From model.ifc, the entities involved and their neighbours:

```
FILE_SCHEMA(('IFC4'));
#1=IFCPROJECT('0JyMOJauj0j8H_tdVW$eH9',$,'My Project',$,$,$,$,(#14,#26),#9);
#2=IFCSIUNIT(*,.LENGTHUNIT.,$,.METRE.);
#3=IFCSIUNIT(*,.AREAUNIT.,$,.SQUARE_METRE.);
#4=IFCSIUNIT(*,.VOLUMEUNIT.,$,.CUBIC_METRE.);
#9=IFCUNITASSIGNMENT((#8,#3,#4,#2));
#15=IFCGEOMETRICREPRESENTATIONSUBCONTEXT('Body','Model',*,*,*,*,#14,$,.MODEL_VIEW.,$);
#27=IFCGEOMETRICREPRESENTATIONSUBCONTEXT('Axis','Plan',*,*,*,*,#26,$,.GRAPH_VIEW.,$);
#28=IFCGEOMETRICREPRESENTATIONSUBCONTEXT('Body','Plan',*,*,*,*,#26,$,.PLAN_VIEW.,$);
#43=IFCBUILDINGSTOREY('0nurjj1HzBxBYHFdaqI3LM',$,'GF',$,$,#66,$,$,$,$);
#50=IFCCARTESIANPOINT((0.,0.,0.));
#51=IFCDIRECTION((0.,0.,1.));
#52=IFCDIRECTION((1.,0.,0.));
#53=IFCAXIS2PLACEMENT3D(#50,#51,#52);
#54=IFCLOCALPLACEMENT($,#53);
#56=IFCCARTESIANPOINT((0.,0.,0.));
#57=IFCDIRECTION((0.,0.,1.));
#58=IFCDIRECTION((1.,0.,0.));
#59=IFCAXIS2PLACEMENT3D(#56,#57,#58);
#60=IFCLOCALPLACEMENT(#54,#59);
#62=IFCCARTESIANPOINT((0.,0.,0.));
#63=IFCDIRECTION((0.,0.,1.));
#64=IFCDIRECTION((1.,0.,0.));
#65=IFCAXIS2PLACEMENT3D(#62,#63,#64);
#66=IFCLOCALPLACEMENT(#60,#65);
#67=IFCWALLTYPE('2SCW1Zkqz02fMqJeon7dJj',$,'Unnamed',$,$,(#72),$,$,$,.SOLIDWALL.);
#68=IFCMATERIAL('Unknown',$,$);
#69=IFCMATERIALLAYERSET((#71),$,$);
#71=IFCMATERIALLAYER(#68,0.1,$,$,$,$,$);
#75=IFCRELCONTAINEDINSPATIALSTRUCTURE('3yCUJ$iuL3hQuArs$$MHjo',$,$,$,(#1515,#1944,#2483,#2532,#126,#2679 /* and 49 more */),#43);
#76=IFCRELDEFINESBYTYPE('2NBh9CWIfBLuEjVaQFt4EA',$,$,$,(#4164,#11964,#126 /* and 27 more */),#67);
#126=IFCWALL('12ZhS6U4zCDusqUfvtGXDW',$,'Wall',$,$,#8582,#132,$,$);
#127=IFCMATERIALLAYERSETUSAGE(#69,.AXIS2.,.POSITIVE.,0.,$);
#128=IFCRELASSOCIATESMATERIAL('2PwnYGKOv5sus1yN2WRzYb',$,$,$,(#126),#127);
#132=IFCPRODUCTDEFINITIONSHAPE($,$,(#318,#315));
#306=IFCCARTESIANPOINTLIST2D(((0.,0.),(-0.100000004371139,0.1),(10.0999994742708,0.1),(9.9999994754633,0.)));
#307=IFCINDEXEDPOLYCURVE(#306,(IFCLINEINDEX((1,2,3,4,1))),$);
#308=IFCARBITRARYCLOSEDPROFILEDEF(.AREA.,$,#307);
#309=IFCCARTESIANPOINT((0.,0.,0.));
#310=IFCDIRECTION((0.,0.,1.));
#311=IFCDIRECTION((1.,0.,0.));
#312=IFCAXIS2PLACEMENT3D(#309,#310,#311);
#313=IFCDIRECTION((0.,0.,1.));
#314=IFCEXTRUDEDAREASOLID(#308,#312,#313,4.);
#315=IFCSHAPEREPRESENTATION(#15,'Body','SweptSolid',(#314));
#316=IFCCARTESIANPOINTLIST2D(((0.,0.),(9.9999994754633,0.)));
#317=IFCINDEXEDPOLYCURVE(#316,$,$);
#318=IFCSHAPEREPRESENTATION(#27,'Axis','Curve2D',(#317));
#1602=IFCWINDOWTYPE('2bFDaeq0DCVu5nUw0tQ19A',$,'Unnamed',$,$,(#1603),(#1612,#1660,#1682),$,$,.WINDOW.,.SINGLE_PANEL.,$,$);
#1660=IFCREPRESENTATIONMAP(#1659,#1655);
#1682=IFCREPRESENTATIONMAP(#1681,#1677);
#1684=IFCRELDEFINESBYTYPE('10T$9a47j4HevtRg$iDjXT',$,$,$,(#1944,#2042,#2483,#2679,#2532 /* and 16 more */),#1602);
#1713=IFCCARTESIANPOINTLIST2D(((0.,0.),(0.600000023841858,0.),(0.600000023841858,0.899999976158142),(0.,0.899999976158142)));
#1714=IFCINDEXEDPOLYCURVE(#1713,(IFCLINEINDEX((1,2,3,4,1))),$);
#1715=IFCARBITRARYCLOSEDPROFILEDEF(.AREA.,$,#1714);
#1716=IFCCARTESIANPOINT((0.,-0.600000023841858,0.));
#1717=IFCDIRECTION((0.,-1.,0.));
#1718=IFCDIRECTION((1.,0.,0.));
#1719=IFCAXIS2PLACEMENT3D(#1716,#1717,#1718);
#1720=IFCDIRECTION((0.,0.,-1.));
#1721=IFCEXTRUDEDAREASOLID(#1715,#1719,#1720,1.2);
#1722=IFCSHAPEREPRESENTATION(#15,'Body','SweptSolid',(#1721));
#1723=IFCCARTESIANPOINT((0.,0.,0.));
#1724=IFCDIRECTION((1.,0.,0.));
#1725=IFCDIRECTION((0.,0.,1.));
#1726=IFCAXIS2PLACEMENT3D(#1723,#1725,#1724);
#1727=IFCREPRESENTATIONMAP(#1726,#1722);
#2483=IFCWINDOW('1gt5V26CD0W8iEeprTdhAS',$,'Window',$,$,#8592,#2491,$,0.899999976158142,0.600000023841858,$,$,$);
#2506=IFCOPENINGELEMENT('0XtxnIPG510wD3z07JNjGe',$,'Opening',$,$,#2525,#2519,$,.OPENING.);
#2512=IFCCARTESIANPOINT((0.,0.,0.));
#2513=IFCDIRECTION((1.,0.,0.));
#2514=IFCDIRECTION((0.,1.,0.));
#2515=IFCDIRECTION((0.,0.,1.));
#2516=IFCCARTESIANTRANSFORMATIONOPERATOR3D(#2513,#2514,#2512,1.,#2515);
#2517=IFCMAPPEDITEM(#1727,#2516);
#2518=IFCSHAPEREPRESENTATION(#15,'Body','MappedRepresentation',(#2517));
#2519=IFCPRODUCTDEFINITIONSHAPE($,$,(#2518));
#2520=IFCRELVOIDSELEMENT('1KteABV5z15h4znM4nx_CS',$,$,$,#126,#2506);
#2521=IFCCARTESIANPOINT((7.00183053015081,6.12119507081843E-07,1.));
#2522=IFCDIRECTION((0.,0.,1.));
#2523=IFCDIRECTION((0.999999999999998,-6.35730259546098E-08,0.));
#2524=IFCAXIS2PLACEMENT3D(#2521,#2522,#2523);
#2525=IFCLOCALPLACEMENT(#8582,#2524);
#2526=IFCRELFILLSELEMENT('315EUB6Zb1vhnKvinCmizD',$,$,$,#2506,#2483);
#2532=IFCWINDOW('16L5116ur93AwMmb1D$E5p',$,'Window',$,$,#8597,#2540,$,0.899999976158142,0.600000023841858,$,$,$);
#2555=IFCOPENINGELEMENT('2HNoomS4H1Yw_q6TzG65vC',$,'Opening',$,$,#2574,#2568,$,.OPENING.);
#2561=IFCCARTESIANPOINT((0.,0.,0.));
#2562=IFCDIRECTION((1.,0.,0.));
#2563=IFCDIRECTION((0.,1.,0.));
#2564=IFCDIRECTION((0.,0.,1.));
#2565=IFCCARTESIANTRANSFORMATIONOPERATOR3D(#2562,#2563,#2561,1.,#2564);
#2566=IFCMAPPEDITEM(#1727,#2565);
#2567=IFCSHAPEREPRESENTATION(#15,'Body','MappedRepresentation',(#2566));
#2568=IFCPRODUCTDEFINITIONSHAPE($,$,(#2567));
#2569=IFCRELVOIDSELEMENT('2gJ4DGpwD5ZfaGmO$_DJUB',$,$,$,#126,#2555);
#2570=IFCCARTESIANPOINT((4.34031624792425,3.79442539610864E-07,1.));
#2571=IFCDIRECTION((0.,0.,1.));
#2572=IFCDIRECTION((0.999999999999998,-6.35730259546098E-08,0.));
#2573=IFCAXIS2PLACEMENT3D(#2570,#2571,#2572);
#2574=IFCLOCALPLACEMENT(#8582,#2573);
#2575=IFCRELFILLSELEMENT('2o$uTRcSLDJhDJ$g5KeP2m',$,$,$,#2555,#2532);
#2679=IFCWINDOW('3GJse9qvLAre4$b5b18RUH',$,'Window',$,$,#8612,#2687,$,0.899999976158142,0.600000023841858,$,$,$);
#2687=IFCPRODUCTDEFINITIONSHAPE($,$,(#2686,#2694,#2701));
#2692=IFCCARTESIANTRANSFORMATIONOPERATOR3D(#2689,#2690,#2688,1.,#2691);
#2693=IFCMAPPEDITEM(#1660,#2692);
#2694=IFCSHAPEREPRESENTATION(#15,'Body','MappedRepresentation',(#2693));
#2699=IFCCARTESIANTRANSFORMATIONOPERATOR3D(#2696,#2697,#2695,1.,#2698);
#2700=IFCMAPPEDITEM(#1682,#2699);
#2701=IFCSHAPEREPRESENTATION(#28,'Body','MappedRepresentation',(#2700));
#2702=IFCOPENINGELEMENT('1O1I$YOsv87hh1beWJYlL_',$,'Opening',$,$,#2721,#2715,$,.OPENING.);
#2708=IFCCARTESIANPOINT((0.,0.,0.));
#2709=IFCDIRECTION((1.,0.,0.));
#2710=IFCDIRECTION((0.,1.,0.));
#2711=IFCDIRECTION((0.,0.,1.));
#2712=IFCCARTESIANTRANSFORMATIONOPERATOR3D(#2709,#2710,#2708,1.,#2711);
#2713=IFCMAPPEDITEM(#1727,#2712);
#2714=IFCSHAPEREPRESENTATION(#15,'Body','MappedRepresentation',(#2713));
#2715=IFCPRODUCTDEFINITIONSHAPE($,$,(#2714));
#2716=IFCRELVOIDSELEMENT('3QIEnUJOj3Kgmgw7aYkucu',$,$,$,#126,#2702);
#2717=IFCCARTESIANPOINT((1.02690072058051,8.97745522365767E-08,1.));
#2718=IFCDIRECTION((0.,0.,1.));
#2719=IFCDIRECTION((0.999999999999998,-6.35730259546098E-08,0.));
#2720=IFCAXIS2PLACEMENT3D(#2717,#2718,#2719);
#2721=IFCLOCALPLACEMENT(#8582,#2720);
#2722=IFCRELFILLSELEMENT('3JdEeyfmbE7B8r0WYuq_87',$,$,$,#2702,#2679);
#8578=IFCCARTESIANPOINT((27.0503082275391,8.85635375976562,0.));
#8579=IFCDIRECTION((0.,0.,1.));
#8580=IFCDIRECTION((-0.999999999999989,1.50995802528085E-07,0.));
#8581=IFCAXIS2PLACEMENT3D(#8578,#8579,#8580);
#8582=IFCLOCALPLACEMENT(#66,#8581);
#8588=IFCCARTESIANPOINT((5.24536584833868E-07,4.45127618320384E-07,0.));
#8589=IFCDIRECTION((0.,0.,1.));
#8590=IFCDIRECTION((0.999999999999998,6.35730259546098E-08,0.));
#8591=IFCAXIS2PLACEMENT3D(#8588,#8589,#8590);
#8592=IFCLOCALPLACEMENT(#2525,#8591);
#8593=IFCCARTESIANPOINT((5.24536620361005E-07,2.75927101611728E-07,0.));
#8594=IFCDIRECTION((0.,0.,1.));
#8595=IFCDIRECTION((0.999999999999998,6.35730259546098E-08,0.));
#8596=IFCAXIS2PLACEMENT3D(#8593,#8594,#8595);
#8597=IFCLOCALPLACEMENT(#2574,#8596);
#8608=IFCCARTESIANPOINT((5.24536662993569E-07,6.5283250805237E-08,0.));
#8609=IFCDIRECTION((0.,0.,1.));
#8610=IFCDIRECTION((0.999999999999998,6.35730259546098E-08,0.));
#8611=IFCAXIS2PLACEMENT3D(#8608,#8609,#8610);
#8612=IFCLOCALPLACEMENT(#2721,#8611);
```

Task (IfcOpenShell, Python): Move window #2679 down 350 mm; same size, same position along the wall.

```python
import numpy as np
import ifcopenshell
import ifcopenshell.api.geometry
import ifcopenshell.util.placement
import ifcopenshell.util.unit

model = ifcopenshell.open("model.ifc")
unit_scale = ifcopenshell.util.unit.calculate_unit_scale(model)

window = model.by_id(2679)
opening = window.FillsVoids[0].RelatingOpeningElement
dz = -0.35 / unit_scale

shift = np.array([0.0, 0.0, dz])
# The window is placed relative to its opening, so it follows when the opening moves.
matrix = ifcopenshell.util.placement.get_local_placement(opening.ObjectPlacement)
matrix[:3, 3] += shift
ifcopenshell.api.geometry.edit_object_placement(
    model, product=opening, matrix=matrix, is_si=False, should_transform_children=True
)

print(f"moved by {dz * unit_scale:+.3f} m")

model.write("model_edited.ifc")
```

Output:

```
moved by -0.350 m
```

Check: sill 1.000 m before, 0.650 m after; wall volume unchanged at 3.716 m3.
